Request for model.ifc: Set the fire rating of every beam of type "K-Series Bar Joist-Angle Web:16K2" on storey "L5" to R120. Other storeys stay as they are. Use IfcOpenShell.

First a look at what the model holds.

```python
import ifcopenshell
import ifcopenshell.util.element

model = ifcopenshell.open("model.ifc")
print(model.schema)
storey = next(s for s in model.by_type("IfcBuildingStorey") if s.Name == "L5")
beams = [e for e in ifcopenshell.util.element.get_decomposition(storey) if e.is_a("IfcBeam")]
seen = {}
for e in beams:
    element_type = ifcopenshell.util.element.get_type(e)
    key = (element_type.Name if element_type != e and element_type else None, ifcopenshell.util.element.get_pset(e, "Pset_BeamCommon", "FireRating"))
    seen[key] = seen.get(key, 0) + 1
for (name, value), count in sorted(seen.items(), key=str):
    print(count, "x", name, "|", value)
```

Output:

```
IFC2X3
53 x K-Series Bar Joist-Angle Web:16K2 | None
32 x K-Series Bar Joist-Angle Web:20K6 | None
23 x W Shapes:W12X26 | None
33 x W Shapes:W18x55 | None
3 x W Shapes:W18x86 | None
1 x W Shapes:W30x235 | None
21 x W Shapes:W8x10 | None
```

```python
import ifcopenshell
import ifcopenshell.api.pset
import ifcopenshell.util.element

model = ifcopenshell.open("model.ifc")

storey = next(s for s in model.by_type("IfcBuildingStorey") if s.Name == "L5")
beams = [e for e in ifcopenshell.util.element.get_decomposition(storey) if e.is_a("IfcBeam")]

count = 0
for e in beams:
    element_type = ifcopenshell.util.element.get_type(e)
    if element_type in (None, e) or element_type.Name != "K-Series Bar Joist-Angle Web:16K2":
        continue
    # add_pset returns the element's existing set when there is one.
    pset = ifcopenshell.api.pset.add_pset(model, product=e, name="Pset_BeamCommon")
    ifcopenshell.api.pset.edit_pset(model, pset=pset, properties={"FireRating": "R120"})
    count += 1

print(count, "beams updated")

model.write("model_edited.ifc")
```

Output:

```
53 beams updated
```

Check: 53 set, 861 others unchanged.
